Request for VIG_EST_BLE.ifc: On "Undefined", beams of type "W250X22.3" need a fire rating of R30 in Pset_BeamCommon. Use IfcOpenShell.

First a look at what the model holds.

```python
import ifcopenshell
import ifcopenshell.util.element

model = ifcopenshell.open("VIG_EST_BLE.ifc")
print(model.schema)
storey = next(s for s in model.by_type("IfcBuildingStorey") if s.Name == "Undefined")
beams = [e for e in ifcopenshell.util.element.get_decomposition(storey) if e.is_a("IfcBeam")]
seen = {}
for e in beams:
    element_type = ifcopenshell.util.element.get_type(e)
    key = (element_type.Name if element_type != e and element_type else None, ifcopenshell.util.element.get_pset(e, "Pset_BeamCommon", "FireRating"))
    seen[key] = seen.get(key, 0) + 1
for (name, value), count in sorted(seen.items(), key=str):
    print(count, "x", name, "|", value)
```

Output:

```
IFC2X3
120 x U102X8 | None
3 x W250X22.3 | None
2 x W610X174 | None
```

```python
import ifcopenshell
import ifcopenshell.api.pset
import ifcopenshell.util.element

model = ifcopenshell.open("VIG_EST_BLE.ifc")

storey = next(s for s in model.by_type("IfcBuildingStorey") if s.Name == "Undefined")
beams = [e for e in ifcopenshell.util.element.get_decomposition(storey) if e.is_a("IfcBeam")]

count = 0
for e in beams:
    element_type = ifcopenshell.util.element.get_type(e)
    if element_type in (None, e) or element_type.Name != "W250X22.3":
        continue
    found = ifcopenshell.util.element.get_pset(e, "Pset_BeamCommon", should_inherit=False)
    if found:
        pset = model.by_id(found["id"])
        if len(ifcopenshell.util.element.get_elements_by_pset(pset)) > 1:
            pset = ifcopenshell.api.pset.unshare_pset(model, products=[e], pset=pset)[0]
    else:
        pset = ifcopenshell.api.pset.add_pset(model, product=e, name="Pset_BeamCommon")
    ifcopenshell.api.pset.edit_pset(model, pset=pset, properties={"FireRating": "R30"})
    count += 1

print(count, "beams updated")

model.write("VIG_EST_BLE_rev.ifc")
```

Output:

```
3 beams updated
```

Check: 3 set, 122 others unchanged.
